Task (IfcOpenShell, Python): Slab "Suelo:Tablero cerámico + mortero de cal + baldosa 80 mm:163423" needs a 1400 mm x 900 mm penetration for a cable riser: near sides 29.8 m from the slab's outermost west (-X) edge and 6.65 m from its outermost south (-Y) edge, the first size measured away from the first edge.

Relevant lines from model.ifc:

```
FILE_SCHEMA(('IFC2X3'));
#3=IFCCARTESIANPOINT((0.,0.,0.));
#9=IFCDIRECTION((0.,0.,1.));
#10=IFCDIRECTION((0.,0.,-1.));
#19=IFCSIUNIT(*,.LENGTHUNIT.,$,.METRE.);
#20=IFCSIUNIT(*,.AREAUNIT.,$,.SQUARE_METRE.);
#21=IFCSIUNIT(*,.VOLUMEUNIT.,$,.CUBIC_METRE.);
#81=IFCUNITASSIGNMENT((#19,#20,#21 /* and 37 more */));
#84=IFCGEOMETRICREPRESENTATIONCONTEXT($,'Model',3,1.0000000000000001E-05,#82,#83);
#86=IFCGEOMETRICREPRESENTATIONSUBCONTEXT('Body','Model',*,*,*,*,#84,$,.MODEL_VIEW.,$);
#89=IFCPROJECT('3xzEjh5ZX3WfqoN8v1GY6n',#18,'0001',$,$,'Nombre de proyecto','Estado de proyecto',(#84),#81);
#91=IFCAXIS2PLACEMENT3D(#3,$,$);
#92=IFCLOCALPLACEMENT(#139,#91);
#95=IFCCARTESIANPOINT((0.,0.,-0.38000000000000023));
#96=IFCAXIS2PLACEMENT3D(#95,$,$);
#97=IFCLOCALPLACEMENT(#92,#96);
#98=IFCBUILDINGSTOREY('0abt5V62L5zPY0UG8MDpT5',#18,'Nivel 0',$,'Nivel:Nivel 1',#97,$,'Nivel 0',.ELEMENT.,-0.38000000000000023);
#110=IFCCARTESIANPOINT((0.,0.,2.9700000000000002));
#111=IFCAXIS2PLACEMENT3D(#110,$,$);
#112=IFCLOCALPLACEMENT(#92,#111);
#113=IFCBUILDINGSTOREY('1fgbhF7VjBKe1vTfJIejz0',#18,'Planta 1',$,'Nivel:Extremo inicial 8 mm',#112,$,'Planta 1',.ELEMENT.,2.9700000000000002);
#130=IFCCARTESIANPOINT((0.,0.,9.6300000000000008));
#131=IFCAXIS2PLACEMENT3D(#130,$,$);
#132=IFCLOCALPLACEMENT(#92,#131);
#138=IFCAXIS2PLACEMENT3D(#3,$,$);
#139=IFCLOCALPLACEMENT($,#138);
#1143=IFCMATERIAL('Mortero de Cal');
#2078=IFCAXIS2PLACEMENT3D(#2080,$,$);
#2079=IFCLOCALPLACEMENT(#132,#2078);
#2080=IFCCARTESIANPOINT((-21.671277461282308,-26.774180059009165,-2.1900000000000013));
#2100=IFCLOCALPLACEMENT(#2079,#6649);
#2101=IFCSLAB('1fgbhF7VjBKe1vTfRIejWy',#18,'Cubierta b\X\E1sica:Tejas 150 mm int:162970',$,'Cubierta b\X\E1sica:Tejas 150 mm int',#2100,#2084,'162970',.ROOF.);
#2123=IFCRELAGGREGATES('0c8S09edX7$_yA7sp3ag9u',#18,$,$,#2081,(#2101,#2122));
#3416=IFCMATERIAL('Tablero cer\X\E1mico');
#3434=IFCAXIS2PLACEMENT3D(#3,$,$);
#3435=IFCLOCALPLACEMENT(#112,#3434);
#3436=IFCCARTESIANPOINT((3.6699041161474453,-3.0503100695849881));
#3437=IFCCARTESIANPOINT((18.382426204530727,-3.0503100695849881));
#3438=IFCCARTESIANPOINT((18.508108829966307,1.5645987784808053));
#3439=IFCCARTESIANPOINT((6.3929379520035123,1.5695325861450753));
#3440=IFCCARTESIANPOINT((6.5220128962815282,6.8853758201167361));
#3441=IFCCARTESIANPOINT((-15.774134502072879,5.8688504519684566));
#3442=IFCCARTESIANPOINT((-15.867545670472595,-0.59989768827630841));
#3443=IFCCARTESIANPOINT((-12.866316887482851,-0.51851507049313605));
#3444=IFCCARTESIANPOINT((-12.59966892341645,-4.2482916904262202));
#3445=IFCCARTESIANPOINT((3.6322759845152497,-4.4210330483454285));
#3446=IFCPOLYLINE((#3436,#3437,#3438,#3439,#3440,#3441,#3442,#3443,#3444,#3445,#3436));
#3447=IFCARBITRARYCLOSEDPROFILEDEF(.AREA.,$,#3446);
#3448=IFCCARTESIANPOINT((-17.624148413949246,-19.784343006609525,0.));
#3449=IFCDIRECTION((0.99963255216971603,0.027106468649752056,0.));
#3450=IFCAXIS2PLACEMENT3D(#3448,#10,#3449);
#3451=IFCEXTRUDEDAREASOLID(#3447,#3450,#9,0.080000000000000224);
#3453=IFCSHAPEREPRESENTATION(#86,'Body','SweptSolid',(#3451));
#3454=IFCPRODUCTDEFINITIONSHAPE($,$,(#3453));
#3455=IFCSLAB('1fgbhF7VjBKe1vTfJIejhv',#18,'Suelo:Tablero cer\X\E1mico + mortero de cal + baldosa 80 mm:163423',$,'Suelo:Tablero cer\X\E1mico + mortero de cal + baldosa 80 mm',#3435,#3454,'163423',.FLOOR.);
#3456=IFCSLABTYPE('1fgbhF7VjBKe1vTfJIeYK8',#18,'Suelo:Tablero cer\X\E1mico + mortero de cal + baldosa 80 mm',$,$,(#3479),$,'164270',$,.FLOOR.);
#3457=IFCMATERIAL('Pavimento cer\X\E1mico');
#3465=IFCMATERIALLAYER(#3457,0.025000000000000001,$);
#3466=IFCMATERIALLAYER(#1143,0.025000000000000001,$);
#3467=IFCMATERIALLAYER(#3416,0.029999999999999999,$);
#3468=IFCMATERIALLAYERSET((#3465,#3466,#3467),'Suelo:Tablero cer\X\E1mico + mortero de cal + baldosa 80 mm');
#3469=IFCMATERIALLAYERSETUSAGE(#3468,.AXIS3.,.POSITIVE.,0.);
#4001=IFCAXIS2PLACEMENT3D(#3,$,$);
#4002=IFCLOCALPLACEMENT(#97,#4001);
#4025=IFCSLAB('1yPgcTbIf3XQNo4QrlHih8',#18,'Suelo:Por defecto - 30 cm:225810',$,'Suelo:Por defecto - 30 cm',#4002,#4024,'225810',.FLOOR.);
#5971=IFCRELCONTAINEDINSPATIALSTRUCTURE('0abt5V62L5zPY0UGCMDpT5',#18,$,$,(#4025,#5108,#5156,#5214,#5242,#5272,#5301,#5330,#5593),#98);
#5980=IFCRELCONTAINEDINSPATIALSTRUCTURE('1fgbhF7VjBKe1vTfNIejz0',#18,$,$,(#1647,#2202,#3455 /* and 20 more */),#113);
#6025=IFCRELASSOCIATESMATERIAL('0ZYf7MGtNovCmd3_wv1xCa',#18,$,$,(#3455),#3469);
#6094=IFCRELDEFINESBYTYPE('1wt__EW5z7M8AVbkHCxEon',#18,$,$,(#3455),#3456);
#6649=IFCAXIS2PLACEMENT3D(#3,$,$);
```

```python
import numpy as np
import ifcopenshell
import ifcopenshell.api.feature
import ifcopenshell.api.geometry
import ifcopenshell.api.root
import ifcopenshell.geom
import ifcopenshell.util.placement
import ifcopenshell.util.representation
import ifcopenshell.util.shape
import ifcopenshell.util.unit

model = ifcopenshell.open("model.ifc")
unit_scale = ifcopenshell.util.unit.calculate_unit_scale(model)
settings = ifcopenshell.geom.settings()


def volume(element):
    """Net volume in cubic metres, openings subtracted."""
    shape = ifcopenshell.geom.create_shape(settings, element)
    return ifcopenshell.util.shape.get_volume(shape.geometry)


slab = model.by_guid("1fgbhF7VjBKe1vTfJIejhv")
before = volume(slab)

# Extent in the slab's own axes, in metres. The edges named are its -X and -Y sides.
slab_shape = ifcopenshell.geom.create_shape(settings, slab)
vertices = ifcopenshell.util.shape.get_vertices(slab_shape.geometry)
x_min, y_min, bottom = vertices.min(axis=0)
top = vertices[:, 2].max()

opening = ifcopenshell.api.root.create_entity(model, ifc_class="IfcOpeningElement", name="Cable riser opening")
context = ifcopenshell.util.representation.get_context(model, "Model", "Body", "MODEL_VIEW")
width, depth = 1.4, 0.9
outline = [(0.0, 0.0), (width, 0.0), (width, depth), (0.0, depth), (0.0, 0.0)]
# Overshoot both faces by 50 mm so the cut is clean.
shape = ifcopenshell.api.geometry.add_slab_representation(
    model, context=context, depth=top - bottom + 0.1, polyline=outline
)
ifcopenshell.api.geometry.assign_representation(model, product=opening, representation=shape)

matrix = ifcopenshell.util.placement.get_local_placement(slab.ObjectPlacement)
matrix[:, 3] = matrix @ np.append(np.array([x_min + 29.8, y_min + 6.65, bottom - 0.05]) / unit_scale, 1.0)
ifcopenshell.api.geometry.edit_object_placement(model, product=opening, matrix=matrix, is_si=False)
ifcopenshell.api.feature.add_feature(model, feature=opening, element=slab)

after = volume(slab)

print(f"slab volume {before:.3f} -> {after:.3f} m3")

model.write("model_rev.ifc")
```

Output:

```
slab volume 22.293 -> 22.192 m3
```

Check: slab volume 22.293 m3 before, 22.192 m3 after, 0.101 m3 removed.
